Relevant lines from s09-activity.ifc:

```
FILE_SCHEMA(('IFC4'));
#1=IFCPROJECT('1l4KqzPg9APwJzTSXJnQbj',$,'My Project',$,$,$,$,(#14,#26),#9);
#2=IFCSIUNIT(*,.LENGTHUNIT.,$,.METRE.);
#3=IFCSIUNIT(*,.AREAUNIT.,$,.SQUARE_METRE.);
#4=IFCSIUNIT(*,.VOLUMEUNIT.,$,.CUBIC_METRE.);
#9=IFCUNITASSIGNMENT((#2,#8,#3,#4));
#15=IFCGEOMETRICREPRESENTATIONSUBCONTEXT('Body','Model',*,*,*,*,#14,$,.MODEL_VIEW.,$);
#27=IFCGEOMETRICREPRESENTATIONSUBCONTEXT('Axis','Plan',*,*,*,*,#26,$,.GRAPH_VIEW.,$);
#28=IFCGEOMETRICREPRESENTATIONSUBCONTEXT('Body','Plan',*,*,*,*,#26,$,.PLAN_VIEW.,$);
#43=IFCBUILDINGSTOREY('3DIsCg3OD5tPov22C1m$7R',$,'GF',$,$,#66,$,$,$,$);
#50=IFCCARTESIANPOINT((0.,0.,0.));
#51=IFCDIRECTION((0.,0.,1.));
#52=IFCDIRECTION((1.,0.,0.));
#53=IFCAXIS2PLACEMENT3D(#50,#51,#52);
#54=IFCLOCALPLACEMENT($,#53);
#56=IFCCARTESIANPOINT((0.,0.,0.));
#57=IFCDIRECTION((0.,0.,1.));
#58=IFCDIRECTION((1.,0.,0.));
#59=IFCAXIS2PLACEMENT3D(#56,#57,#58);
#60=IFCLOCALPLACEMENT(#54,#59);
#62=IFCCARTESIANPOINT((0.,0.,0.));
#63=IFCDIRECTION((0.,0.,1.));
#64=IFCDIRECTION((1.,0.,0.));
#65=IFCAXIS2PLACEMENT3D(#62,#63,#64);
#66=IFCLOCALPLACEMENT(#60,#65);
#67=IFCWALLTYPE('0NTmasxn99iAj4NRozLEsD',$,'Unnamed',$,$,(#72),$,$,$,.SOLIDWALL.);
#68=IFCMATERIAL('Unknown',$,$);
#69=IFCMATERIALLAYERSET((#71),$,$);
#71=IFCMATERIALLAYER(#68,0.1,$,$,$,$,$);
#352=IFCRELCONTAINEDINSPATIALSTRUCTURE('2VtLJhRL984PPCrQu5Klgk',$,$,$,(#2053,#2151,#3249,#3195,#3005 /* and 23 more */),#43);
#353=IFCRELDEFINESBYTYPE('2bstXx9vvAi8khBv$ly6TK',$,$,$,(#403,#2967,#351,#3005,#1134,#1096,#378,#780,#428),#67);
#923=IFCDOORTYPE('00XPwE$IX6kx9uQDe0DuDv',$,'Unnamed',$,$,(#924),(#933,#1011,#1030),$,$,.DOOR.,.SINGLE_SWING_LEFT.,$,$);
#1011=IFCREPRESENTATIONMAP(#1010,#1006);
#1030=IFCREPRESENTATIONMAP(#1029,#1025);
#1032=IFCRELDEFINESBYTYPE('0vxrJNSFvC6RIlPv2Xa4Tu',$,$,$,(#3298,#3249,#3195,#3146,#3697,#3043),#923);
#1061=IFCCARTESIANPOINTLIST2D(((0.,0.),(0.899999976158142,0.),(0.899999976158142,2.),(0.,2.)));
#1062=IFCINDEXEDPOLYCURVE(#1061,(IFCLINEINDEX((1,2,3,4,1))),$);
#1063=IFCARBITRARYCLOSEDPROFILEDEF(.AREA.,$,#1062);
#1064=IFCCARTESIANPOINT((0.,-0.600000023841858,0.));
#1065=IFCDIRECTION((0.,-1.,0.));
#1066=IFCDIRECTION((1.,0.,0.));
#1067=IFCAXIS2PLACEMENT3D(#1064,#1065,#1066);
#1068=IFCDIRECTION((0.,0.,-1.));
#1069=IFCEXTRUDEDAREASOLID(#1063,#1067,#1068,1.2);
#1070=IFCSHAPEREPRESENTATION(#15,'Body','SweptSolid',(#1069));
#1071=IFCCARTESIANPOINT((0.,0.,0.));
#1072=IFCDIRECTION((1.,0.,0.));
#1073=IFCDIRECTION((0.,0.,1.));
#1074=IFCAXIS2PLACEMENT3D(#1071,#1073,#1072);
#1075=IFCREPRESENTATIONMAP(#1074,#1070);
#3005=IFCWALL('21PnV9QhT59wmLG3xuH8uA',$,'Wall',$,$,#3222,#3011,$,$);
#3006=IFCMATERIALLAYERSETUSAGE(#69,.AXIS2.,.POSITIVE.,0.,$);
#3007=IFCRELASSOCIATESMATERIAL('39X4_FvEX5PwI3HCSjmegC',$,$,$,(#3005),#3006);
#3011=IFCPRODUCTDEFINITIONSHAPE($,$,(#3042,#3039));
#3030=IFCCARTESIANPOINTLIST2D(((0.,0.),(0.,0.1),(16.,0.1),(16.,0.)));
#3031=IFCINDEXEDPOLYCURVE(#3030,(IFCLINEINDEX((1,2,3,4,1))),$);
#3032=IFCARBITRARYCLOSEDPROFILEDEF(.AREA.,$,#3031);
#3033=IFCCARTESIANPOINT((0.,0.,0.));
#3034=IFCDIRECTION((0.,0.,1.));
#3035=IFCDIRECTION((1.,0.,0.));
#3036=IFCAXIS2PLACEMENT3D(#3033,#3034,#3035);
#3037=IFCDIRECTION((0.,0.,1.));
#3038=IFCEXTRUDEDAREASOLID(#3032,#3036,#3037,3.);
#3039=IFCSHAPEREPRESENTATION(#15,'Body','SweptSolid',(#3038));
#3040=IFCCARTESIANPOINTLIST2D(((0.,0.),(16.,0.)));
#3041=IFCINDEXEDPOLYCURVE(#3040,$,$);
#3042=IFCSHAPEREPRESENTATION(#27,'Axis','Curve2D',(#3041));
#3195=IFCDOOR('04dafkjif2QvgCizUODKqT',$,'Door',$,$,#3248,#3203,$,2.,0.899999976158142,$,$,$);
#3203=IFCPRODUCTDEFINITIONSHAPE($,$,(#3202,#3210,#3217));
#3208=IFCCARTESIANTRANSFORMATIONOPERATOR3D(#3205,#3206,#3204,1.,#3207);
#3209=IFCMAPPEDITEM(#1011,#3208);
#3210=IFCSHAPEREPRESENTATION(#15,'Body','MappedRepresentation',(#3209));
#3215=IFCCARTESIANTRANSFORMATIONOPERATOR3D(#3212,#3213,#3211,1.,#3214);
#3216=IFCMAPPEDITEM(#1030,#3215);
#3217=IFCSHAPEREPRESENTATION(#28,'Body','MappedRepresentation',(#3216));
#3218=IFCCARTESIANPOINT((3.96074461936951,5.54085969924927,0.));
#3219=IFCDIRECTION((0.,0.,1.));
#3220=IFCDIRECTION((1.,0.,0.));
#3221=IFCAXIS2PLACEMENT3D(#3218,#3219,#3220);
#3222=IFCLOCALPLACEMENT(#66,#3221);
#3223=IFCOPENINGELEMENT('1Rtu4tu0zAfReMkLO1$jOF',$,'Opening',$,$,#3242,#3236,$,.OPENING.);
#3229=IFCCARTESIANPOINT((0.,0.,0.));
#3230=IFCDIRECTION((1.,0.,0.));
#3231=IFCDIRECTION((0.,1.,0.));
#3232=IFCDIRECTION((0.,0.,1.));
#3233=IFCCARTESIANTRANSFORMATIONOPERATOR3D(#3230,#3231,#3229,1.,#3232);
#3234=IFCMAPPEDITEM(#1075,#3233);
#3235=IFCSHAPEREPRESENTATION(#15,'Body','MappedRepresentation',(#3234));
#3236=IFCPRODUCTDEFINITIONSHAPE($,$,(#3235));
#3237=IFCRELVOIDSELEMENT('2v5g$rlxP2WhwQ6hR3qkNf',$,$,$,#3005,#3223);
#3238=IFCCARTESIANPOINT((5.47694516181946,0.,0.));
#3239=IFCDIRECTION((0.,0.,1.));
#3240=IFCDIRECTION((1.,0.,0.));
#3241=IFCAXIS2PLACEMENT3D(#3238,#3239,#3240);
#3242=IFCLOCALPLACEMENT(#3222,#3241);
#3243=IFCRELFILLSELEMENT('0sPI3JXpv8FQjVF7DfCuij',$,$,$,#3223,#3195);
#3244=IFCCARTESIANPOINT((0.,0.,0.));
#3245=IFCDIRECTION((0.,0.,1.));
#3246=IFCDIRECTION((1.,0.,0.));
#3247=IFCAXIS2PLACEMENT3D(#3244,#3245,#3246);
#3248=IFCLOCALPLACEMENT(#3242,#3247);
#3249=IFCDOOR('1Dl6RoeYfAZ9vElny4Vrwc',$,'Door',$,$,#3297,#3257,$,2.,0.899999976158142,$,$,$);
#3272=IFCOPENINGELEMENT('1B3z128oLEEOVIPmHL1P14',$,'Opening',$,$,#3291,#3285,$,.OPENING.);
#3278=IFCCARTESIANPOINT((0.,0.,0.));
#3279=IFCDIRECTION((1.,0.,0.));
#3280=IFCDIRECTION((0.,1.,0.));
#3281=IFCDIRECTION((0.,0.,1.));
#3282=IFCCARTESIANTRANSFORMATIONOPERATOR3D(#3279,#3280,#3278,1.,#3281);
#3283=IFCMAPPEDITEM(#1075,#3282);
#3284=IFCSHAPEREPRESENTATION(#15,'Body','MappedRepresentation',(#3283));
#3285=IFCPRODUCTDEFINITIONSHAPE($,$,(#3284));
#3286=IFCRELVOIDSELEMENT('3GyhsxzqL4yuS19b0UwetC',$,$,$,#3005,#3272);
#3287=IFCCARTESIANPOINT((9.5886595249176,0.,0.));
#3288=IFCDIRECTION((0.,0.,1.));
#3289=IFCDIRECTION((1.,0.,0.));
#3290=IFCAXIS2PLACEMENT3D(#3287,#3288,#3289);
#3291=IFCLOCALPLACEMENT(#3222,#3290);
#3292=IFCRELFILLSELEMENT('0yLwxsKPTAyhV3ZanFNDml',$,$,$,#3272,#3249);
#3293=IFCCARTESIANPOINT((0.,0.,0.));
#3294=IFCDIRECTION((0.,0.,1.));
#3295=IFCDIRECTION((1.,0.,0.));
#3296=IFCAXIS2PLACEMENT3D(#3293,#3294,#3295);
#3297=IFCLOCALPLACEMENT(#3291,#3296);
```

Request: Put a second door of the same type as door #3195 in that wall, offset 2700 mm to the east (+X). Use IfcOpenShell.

```python
import ifcopenshell
import ifcopenshell.api.feature
import ifcopenshell.api.geometry
import ifcopenshell.api.root
import ifcopenshell.geom
import ifcopenshell.util.element
import ifcopenshell.util.placement
import ifcopenshell.util.shape

model = ifcopenshell.open("s09-activity.ifc")
settings = ifcopenshell.geom.settings()


def volume(element):
    """Net volume in cubic metres, openings subtracted."""
    shape = ifcopenshell.geom.create_shape(settings, element)
    return ifcopenshell.util.shape.get_volume(shape.geometry)


door = model.by_id(3195)
opening = door.FillsVoids[0].RelatingOpeningElement
wall = opening.VoidsElements[0].RelatingBuildingElement
before = volume(wall)
shift = ifcopenshell.util.placement.get_local_placement(wall.ObjectPlacement)[:3, 0] * 2.7

# copy_class copies the void relationship, type, container and properties, but no geometry.
new_opening = ifcopenshell.api.root.copy_class(model, product=opening)
new_opening.Representation = ifcopenshell.util.element.copy_deep(
    model, opening.Representation, exclude=["IfcGeometricRepresentationContext", "IfcRepresentationMap"]
)
new_door = ifcopenshell.api.root.copy_class(model, product=door)
new_door.Representation = ifcopenshell.util.element.copy_deep(
    model, door.Representation, exclude=["IfcGeometricRepresentationContext", "IfcRepresentationMap"]
)
ifcopenshell.api.feature.add_filling(model, opening=new_opening, element=new_door)

for old, new in ((opening, new_opening), (door, new_door)):
    matrix = ifcopenshell.util.placement.get_local_placement(old.ObjectPlacement)
    matrix[:3, 3] += shift
    ifcopenshell.api.geometry.edit_object_placement(model, product=new, matrix=matrix, is_si=False)

after = volume(wall)

print(f"wall volume {before:.3f} -> {after:.3f} m3")

model.write("s09-activity-out.ifc")
```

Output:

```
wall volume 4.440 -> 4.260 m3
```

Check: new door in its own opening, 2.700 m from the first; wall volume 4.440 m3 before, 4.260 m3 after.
